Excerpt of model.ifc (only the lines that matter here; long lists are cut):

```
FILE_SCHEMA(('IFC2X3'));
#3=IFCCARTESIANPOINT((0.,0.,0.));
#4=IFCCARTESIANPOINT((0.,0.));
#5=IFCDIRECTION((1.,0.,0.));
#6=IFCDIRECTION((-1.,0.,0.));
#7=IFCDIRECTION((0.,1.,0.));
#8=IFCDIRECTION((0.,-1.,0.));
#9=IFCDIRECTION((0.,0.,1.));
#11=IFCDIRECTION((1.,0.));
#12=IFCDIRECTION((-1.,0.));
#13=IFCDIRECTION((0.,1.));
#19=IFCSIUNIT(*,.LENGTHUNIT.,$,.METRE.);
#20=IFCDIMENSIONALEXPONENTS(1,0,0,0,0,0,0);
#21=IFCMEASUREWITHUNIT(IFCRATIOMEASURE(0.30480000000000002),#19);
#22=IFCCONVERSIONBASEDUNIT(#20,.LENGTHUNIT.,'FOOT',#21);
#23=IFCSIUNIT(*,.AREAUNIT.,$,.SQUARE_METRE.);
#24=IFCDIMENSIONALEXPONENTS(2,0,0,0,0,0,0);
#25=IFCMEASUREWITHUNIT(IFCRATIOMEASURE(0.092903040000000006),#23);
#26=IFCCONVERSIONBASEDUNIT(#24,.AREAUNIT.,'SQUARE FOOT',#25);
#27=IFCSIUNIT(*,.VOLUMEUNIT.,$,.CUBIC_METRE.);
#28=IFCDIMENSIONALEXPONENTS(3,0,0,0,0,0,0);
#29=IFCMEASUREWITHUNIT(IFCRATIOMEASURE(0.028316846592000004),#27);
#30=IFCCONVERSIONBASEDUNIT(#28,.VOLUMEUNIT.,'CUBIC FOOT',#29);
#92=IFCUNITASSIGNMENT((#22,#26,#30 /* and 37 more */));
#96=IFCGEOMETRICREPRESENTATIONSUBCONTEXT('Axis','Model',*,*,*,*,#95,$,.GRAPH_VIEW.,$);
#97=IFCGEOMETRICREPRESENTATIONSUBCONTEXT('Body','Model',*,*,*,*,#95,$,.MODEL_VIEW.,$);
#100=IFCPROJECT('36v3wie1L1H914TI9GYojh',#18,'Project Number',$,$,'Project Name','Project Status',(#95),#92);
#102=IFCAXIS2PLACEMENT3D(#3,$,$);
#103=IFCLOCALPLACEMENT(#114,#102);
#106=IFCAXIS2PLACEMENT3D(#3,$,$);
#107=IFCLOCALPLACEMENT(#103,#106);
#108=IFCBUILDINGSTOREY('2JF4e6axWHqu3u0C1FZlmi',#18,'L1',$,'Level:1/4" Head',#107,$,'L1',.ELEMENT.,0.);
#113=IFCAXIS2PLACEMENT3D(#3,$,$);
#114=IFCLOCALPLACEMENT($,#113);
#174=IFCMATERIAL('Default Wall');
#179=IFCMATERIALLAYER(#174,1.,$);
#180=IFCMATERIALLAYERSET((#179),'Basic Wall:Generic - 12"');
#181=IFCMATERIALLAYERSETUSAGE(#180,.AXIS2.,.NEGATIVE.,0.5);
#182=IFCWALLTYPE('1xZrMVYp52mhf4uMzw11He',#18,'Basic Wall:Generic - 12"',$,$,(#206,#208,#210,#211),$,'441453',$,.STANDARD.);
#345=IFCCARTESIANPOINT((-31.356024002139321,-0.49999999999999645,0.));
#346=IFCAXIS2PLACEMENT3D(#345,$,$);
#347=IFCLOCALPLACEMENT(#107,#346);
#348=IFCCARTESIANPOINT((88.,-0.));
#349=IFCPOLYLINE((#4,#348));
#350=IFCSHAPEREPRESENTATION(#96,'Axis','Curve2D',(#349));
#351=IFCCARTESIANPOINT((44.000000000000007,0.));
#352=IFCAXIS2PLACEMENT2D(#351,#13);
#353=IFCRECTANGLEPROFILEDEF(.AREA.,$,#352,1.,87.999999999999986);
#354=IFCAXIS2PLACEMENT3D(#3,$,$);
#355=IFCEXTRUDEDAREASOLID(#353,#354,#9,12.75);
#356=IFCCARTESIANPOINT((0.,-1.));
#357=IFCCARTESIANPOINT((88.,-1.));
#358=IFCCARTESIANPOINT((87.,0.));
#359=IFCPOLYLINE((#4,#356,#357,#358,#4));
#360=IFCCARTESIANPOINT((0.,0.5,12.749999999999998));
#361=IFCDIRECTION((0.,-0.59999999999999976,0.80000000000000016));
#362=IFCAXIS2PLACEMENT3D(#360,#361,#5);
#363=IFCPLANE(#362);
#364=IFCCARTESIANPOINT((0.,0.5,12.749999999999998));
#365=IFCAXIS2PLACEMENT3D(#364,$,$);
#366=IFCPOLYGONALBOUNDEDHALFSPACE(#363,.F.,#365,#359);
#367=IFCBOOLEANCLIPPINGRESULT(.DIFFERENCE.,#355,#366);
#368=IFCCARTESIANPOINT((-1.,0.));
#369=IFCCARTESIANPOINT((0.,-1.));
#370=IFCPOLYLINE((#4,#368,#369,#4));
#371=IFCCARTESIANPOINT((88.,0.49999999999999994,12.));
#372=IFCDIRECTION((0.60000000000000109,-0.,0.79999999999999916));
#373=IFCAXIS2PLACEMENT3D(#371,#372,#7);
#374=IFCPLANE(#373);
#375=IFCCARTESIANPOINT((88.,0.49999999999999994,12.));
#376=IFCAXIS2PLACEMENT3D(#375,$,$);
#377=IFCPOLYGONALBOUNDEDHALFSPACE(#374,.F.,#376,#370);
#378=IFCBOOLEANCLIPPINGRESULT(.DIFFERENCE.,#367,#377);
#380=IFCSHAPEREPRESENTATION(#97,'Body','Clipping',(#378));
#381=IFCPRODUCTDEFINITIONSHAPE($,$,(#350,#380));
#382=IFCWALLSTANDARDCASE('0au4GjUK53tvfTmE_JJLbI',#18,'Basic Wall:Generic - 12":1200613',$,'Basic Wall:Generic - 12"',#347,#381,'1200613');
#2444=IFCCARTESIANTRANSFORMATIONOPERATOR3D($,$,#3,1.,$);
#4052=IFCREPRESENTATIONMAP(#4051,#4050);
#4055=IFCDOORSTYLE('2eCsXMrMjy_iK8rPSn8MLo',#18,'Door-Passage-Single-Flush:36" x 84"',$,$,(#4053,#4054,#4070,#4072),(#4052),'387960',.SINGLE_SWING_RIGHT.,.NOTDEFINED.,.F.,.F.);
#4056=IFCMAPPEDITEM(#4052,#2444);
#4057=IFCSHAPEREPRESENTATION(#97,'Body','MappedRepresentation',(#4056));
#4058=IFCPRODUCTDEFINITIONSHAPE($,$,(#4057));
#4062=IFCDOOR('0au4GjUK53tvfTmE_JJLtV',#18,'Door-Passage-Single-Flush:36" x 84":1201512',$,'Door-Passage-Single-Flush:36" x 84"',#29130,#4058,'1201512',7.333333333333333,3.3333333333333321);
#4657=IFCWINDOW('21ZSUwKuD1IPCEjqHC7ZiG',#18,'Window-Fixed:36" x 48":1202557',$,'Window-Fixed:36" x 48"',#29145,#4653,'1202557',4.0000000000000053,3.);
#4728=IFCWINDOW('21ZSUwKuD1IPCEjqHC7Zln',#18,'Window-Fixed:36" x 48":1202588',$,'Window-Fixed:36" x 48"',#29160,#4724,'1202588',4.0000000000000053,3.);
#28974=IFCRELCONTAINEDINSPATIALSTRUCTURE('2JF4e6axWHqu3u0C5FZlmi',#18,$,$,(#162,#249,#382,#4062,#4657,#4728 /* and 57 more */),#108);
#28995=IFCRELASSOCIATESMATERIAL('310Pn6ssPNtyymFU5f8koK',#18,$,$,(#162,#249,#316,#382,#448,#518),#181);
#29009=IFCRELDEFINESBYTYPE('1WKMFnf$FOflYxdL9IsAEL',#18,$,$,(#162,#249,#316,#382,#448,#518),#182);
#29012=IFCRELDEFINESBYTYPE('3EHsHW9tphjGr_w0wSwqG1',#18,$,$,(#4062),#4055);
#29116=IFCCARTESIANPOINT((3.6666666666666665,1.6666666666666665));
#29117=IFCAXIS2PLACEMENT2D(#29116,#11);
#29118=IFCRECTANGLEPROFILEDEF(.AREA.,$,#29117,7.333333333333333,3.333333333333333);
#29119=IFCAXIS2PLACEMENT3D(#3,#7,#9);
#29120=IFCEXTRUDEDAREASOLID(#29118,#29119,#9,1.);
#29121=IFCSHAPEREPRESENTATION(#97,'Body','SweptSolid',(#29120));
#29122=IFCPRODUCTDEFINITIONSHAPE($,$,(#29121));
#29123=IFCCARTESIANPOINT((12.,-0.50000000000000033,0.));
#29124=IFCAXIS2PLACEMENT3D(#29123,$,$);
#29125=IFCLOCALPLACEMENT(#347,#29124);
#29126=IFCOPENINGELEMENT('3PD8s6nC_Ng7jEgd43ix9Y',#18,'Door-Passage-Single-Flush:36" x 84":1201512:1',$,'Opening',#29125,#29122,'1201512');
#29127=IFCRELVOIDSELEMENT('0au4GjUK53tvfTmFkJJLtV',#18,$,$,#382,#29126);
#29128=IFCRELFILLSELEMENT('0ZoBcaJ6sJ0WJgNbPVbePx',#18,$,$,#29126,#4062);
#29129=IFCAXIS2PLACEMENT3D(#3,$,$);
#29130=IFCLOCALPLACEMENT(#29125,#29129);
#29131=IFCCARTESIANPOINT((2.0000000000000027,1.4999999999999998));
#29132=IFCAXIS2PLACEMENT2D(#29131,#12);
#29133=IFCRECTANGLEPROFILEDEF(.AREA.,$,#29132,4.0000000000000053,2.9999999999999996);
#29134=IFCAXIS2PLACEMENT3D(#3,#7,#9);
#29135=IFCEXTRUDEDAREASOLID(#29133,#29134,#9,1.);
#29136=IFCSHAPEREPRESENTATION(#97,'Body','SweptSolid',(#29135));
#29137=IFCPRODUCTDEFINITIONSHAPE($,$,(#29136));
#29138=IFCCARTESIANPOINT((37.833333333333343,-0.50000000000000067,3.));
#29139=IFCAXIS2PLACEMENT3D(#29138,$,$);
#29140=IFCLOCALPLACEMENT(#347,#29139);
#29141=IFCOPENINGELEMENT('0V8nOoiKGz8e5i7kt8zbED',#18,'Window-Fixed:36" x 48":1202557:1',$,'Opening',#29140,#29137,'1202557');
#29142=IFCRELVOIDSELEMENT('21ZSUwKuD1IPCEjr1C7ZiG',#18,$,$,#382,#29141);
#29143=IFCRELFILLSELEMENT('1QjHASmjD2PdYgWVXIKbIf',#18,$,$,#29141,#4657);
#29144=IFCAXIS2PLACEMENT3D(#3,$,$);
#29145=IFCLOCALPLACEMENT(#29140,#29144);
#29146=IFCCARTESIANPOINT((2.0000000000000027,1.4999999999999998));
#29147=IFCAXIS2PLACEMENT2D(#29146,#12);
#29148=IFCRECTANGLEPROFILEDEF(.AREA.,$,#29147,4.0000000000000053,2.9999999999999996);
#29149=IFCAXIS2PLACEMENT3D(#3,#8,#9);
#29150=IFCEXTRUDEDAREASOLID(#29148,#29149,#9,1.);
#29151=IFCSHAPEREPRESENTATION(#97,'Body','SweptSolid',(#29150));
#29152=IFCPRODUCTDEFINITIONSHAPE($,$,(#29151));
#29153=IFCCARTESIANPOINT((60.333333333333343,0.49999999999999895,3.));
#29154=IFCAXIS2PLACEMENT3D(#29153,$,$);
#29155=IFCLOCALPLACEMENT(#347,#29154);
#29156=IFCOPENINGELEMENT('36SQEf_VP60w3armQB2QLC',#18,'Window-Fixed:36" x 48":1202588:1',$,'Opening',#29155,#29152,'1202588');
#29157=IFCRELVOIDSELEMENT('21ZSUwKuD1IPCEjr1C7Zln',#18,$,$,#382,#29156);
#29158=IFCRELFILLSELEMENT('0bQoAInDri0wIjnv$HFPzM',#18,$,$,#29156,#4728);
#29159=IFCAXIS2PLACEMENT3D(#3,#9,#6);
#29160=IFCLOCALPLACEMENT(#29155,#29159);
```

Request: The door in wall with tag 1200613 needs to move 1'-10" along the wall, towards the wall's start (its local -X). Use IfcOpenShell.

```python
import ifcopenshell
import ifcopenshell.api.geometry
import ifcopenshell.util.placement
import ifcopenshell.util.unit

model = ifcopenshell.open("model.ifc")
unit_scale = ifcopenshell.util.unit.calculate_unit_scale(model)

door = model.by_guid("0au4GjUK53tvfTmE_JJLtV")
opening = door.FillsVoids[0].RelatingOpeningElement
wall = opening.VoidsElements[0].RelatingBuildingElement

wall_matrix = ifcopenshell.util.placement.get_local_placement(wall.ObjectPlacement)
shift = wall_matrix[:3, 0] * -22 * 0.0254 / unit_scale
before = ifcopenshell.util.placement.get_local_placement(door.ObjectPlacement)[:3, 3].copy()

# The door is placed relative to its opening, so it follows when the opening moves.
matrix = ifcopenshell.util.placement.get_local_placement(opening.ObjectPlacement)
matrix[:3, 3] += shift
ifcopenshell.api.geometry.edit_object_placement(
    model, product=opening, matrix=matrix, is_si=False, should_transform_children=True
)

after = ifcopenshell.util.placement.get_local_placement(door.ObjectPlacement)[:3, 3]
print("door moved by", (after - before).round(3) + 0.0)

model.write("model_updated.ifc")
```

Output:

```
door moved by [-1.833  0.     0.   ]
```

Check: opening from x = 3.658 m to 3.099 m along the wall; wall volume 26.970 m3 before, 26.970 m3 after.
